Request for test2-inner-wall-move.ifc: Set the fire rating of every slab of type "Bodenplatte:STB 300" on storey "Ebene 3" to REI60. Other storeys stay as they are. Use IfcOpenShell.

First a look at what the model holds.

```python
import ifcopenshell
import ifcopenshell.util.element

model = ifcopenshell.open("test2-inner-wall-move.ifc")
print(model.schema)
storey = next(s for s in model.by_type("IfcBuildingStorey") if s.Name == "Ebene 3")
slabs = [e for e in ifcopenshell.util.element.get_decomposition(storey) if e.is_a("IfcSlab")]
seen = {}
for e in slabs:
    element_type = ifcopenshell.util.element.get_type(e)
    key = (element_type.Name if element_type != e and element_type else None, ifcopenshell.util.element.get_pset(e, "Pset_SlabCommon", "FireRating"))
    seen[key] = seen.get(key, 0) + 1
for (name, value), count in sorted(seen.items(), key=str):
    print(count, "x", name, "|", value)
```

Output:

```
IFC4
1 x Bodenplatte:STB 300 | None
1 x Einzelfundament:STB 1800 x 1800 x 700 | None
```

```python
import ifcopenshell
import ifcopenshell.api.pset
import ifcopenshell.util.element

model = ifcopenshell.open("test2-inner-wall-move.ifc")

storey = next(s for s in model.by_type("IfcBuildingStorey") if s.Name == "Ebene 3")
slabs = [e for e in ifcopenshell.util.element.get_decomposition(storey) if e.is_a("IfcSlab")]

count = 0
for e in slabs:
    element_type = ifcopenshell.util.element.get_type(e)
    if element_type in (None, e) or element_type.Name != "Bodenplatte:STB 300":
        continue
    # add_pset returns the element's existing set when there is one.
    pset = ifcopenshell.api.pset.add_pset(model, product=e, name="Pset_SlabCommon")
    ifcopenshell.api.pset.edit_pset(model, pset=pset, properties={"FireRating": "REI60"})
    count += 1

print(count, "slabs updated")

model.write("test2-inner-wall-move_updated.ifc")
```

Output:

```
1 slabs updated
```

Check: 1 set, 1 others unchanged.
